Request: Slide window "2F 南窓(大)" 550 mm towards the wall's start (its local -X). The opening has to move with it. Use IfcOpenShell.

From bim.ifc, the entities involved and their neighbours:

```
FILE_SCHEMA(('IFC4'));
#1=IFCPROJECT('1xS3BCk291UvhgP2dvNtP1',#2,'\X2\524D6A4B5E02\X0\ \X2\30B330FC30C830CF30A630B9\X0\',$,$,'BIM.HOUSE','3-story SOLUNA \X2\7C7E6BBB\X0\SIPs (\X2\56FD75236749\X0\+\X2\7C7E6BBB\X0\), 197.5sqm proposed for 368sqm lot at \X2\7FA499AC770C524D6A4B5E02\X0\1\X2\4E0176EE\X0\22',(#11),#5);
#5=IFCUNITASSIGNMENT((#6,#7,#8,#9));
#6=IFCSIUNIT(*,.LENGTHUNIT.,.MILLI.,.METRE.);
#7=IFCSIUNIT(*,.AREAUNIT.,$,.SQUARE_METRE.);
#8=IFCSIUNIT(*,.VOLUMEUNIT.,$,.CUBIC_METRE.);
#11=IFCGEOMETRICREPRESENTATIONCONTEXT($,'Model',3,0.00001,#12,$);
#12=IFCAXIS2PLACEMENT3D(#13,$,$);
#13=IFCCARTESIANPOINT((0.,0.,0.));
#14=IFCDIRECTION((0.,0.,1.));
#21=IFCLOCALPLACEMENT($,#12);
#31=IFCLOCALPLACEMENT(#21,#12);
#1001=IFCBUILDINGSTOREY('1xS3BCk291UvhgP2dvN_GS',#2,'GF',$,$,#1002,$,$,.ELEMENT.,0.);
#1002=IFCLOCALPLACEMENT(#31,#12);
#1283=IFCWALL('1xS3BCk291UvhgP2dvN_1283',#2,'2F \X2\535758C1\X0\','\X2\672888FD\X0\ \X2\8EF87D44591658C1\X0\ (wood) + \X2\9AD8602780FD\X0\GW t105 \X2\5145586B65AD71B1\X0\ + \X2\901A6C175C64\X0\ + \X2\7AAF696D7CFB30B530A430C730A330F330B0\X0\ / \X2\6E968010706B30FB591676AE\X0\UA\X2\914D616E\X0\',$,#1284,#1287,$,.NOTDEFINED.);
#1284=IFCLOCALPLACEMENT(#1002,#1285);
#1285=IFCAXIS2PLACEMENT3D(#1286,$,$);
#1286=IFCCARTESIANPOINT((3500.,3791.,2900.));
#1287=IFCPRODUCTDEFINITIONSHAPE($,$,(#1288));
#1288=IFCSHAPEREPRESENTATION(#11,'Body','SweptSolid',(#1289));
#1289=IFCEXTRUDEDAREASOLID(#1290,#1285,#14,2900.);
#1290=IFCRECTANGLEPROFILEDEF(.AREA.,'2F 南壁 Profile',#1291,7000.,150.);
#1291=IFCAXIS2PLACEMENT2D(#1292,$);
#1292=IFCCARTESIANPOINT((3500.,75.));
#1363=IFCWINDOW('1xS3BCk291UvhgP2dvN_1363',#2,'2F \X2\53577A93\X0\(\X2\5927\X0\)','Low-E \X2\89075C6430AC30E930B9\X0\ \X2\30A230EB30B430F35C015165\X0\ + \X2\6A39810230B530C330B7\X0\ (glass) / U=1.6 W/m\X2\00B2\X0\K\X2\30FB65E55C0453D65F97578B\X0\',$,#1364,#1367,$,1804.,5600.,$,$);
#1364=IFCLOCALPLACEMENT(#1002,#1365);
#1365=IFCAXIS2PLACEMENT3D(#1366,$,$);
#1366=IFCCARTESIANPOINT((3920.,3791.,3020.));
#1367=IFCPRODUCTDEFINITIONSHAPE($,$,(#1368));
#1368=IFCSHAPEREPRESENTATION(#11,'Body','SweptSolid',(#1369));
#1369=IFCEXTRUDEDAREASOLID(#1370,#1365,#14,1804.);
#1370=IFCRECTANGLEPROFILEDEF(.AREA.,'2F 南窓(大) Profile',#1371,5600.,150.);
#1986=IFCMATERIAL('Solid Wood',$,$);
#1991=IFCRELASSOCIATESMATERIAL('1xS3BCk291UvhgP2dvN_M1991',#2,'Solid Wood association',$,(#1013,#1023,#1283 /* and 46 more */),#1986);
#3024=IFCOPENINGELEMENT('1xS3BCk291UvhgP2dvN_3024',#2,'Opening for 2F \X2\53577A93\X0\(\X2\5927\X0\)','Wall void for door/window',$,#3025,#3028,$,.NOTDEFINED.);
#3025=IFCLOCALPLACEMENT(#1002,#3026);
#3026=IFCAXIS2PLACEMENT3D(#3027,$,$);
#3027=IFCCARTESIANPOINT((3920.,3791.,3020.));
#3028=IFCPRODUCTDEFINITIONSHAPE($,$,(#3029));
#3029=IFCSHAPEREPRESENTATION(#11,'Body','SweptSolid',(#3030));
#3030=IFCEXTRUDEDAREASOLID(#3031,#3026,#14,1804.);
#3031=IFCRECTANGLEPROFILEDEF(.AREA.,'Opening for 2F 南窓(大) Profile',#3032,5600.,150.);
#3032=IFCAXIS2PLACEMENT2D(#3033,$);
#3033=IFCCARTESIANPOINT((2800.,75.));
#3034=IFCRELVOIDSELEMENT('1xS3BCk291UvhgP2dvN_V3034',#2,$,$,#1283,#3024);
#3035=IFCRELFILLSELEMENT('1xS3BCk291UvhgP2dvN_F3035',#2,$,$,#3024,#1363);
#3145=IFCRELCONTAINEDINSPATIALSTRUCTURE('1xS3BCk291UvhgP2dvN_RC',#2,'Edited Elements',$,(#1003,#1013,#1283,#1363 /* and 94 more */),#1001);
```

```python
import ifcopenshell
import ifcopenshell.api.geometry
import ifcopenshell.util.placement
import ifcopenshell.util.unit

model = ifcopenshell.open("bim.ifc")
unit_scale = ifcopenshell.util.unit.calculate_unit_scale(model)

window = model.by_guid("1xS3BCk291UvhgP2dvN_1363")
opening = window.FillsVoids[0].RelatingOpeningElement
wall = opening.VoidsElements[0].RelatingBuildingElement

wall_matrix = ifcopenshell.util.placement.get_local_placement(wall.ObjectPlacement)
shift = wall_matrix[:3, 0] * -0.55 / unit_scale
before = ifcopenshell.util.placement.get_local_placement(window.ObjectPlacement)[:3, 3].copy()

# The window is not placed relative to its opening, so move both.
for product in (opening, window):
    matrix = ifcopenshell.util.placement.get_local_placement(product.ObjectPlacement)
    matrix[:3, 3] += shift
    ifcopenshell.api.geometry.edit_object_placement(model, product=product, matrix=matrix, is_si=False)

after = ifcopenshell.util.placement.get_local_placement(window.ObjectPlacement)[:3, 3]
print("window moved by", (after - before).round(3) + 0.0)

model.write("bim_v2.ifc")
```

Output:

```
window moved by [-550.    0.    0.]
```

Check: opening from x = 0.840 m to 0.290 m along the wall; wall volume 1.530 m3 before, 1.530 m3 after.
